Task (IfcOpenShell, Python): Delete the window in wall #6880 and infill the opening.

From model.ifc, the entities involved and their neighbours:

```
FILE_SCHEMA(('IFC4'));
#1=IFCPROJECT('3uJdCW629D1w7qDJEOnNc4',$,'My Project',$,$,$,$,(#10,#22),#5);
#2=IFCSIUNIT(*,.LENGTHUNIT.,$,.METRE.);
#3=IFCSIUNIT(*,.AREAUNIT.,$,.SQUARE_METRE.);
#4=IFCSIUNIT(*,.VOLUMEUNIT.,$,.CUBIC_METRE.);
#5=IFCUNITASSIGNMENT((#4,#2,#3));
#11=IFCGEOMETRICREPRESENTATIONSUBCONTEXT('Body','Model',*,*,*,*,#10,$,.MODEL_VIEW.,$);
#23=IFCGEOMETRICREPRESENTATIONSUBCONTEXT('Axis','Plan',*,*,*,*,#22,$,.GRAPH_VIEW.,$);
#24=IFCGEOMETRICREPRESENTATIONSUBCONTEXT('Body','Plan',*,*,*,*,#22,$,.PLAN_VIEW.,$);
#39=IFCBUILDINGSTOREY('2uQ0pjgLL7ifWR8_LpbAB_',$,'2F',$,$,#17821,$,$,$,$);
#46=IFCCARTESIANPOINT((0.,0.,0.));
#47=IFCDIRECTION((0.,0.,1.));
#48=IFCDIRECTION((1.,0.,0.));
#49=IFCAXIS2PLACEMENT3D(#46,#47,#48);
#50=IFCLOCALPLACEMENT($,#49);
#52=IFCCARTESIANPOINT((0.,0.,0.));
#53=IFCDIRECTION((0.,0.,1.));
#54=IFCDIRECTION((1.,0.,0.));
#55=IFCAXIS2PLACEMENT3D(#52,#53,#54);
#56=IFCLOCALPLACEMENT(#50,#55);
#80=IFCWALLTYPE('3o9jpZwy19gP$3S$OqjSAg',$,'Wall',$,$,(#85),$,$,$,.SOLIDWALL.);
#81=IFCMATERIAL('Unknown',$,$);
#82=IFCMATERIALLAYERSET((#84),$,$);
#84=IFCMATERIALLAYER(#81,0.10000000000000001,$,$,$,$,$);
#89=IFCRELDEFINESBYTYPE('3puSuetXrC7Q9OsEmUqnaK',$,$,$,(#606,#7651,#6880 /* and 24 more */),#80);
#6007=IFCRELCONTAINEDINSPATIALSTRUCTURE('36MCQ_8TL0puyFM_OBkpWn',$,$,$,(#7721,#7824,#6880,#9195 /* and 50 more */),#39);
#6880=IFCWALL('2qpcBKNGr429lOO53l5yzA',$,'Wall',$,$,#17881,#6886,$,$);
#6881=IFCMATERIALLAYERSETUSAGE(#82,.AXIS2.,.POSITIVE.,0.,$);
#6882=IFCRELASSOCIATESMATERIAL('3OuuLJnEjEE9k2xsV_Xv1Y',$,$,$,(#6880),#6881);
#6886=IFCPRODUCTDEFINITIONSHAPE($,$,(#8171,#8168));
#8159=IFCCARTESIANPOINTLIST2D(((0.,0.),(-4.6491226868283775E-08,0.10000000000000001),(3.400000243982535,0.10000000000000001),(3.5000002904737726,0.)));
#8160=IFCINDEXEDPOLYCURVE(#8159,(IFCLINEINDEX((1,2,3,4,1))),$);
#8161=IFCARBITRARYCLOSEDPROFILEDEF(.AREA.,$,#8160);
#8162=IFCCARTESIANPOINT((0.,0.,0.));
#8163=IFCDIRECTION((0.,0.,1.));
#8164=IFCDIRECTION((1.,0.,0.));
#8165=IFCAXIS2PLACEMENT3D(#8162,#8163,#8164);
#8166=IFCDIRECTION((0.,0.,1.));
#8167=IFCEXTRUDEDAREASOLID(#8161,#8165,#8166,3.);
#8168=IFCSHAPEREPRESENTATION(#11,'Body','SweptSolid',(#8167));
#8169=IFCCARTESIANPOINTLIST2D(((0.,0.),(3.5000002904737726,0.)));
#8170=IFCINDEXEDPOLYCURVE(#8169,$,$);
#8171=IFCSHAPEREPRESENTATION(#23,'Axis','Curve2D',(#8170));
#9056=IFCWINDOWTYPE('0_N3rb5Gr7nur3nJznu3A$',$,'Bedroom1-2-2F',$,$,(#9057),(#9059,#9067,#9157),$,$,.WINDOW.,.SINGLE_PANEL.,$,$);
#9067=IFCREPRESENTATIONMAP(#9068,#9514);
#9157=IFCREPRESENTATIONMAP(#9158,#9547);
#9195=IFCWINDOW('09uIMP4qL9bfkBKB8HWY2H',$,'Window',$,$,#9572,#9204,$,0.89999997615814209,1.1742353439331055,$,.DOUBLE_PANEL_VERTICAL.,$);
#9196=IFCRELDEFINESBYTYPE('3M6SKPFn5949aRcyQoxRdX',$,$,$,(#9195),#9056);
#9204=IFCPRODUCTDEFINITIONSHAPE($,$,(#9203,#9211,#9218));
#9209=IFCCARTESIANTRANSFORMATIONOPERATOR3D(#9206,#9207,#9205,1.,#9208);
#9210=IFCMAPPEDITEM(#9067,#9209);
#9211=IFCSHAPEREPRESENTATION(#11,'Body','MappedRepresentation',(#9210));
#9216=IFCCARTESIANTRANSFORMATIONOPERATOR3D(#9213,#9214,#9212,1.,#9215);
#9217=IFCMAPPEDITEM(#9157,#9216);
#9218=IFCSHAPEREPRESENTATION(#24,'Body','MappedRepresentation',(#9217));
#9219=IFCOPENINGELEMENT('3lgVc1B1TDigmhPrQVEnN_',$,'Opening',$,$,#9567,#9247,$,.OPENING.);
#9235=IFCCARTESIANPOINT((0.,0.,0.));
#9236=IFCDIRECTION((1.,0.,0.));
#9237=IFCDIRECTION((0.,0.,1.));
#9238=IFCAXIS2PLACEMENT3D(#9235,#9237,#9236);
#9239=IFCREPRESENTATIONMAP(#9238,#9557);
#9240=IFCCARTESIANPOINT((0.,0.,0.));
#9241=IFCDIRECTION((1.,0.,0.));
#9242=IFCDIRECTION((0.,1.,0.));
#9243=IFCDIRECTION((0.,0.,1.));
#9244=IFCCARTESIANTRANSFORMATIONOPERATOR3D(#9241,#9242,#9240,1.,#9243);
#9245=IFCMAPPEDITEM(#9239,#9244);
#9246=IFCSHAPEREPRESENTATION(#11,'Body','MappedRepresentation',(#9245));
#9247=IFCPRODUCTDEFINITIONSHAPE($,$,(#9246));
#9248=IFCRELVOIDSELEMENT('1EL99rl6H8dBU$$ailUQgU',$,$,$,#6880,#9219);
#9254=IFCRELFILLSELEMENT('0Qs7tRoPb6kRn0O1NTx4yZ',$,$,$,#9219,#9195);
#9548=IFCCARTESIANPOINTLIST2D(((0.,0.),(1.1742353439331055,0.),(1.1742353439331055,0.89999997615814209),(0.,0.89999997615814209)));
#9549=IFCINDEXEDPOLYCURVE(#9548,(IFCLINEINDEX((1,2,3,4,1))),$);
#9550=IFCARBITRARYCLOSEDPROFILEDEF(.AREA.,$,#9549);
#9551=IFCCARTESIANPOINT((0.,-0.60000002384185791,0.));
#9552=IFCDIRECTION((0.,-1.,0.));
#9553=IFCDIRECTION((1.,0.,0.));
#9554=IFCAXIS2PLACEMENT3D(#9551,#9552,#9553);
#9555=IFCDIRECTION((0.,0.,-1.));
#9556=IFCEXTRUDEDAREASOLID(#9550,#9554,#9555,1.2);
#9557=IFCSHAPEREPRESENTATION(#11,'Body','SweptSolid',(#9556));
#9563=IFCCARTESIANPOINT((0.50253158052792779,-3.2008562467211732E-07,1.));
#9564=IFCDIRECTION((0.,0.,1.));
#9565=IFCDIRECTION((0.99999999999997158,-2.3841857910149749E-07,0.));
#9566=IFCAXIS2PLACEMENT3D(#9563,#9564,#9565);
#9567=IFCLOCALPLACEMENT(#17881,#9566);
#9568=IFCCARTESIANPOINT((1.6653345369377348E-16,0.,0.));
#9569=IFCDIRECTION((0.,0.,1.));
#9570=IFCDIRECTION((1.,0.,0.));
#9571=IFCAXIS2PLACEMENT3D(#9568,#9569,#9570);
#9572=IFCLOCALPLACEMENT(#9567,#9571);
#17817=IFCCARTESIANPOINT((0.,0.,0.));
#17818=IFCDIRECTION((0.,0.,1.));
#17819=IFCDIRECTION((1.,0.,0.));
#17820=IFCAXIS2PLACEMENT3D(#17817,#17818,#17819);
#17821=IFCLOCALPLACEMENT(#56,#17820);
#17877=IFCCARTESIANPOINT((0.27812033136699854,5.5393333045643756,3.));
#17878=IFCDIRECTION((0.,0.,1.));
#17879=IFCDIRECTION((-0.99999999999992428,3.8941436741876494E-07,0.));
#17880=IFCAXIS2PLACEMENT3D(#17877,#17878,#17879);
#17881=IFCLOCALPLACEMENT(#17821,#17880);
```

```python
import ifcopenshell
import ifcopenshell.api.feature
import ifcopenshell.api.root
import ifcopenshell.geom
import ifcopenshell.util.shape

model = ifcopenshell.open("model.ifc")
settings = ifcopenshell.geom.settings()


def volume(element):
    """Net volume in cubic metres, openings subtracted."""
    shape = ifcopenshell.geom.create_shape(settings, element)
    return ifcopenshell.util.shape.get_volume(shape.geometry)


window = model.by_id(9195)
opening = window.FillsVoids[0].RelatingOpeningElement
wall = opening.VoidsElements[0].RelatingBuildingElement
before = volume(wall)

ifcopenshell.api.root.remove_product(model, product=window)
ifcopenshell.api.feature.remove_feature(model, feature=opening)

after = volume(wall)

print(f"wall volume {before:.3f} -> {after:.3f} m3")

model.write("model-out.ifc")
```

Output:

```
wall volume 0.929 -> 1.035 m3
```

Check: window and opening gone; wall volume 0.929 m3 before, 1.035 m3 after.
